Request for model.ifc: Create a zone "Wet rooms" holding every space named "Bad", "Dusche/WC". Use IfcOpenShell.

First a look at what the model holds.

```python
import ifcopenshell

model = ifcopenshell.open("model.ifc")
print(model.schema)
seen = {}
for space in model.by_type("IfcSpace"):
    seen[space.LongName] = seen.get(space.LongName, 0) + 1
for name, count in sorted(seen.items(), key=str):
    print(count, "x", name)
print("zones:", [z.Name for z in model.by_type("IfcZone")][:20])
```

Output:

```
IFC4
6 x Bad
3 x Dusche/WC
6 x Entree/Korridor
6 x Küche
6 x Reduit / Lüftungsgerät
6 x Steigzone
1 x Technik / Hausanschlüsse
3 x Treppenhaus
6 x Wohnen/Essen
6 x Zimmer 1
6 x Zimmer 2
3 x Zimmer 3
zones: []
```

```python
import ifcopenshell
import ifcopenshell.api.group
import ifcopenshell.api.root

model = ifcopenshell.open("model.ifc")

names = {"Bad", "Dusche/WC"}
spaces = [s for s in model.by_type("IfcSpace") if s.LongName in names]

zone = ifcopenshell.api.root.create_entity(model, ifc_class="IfcZone", name="Wet rooms")
ifcopenshell.api.group.assign_group(model, products=spaces, group=zone)
print(len(spaces), "spaces in", zone.Name)

model.write("model_rev.ifc")
```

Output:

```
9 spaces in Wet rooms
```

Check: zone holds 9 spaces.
